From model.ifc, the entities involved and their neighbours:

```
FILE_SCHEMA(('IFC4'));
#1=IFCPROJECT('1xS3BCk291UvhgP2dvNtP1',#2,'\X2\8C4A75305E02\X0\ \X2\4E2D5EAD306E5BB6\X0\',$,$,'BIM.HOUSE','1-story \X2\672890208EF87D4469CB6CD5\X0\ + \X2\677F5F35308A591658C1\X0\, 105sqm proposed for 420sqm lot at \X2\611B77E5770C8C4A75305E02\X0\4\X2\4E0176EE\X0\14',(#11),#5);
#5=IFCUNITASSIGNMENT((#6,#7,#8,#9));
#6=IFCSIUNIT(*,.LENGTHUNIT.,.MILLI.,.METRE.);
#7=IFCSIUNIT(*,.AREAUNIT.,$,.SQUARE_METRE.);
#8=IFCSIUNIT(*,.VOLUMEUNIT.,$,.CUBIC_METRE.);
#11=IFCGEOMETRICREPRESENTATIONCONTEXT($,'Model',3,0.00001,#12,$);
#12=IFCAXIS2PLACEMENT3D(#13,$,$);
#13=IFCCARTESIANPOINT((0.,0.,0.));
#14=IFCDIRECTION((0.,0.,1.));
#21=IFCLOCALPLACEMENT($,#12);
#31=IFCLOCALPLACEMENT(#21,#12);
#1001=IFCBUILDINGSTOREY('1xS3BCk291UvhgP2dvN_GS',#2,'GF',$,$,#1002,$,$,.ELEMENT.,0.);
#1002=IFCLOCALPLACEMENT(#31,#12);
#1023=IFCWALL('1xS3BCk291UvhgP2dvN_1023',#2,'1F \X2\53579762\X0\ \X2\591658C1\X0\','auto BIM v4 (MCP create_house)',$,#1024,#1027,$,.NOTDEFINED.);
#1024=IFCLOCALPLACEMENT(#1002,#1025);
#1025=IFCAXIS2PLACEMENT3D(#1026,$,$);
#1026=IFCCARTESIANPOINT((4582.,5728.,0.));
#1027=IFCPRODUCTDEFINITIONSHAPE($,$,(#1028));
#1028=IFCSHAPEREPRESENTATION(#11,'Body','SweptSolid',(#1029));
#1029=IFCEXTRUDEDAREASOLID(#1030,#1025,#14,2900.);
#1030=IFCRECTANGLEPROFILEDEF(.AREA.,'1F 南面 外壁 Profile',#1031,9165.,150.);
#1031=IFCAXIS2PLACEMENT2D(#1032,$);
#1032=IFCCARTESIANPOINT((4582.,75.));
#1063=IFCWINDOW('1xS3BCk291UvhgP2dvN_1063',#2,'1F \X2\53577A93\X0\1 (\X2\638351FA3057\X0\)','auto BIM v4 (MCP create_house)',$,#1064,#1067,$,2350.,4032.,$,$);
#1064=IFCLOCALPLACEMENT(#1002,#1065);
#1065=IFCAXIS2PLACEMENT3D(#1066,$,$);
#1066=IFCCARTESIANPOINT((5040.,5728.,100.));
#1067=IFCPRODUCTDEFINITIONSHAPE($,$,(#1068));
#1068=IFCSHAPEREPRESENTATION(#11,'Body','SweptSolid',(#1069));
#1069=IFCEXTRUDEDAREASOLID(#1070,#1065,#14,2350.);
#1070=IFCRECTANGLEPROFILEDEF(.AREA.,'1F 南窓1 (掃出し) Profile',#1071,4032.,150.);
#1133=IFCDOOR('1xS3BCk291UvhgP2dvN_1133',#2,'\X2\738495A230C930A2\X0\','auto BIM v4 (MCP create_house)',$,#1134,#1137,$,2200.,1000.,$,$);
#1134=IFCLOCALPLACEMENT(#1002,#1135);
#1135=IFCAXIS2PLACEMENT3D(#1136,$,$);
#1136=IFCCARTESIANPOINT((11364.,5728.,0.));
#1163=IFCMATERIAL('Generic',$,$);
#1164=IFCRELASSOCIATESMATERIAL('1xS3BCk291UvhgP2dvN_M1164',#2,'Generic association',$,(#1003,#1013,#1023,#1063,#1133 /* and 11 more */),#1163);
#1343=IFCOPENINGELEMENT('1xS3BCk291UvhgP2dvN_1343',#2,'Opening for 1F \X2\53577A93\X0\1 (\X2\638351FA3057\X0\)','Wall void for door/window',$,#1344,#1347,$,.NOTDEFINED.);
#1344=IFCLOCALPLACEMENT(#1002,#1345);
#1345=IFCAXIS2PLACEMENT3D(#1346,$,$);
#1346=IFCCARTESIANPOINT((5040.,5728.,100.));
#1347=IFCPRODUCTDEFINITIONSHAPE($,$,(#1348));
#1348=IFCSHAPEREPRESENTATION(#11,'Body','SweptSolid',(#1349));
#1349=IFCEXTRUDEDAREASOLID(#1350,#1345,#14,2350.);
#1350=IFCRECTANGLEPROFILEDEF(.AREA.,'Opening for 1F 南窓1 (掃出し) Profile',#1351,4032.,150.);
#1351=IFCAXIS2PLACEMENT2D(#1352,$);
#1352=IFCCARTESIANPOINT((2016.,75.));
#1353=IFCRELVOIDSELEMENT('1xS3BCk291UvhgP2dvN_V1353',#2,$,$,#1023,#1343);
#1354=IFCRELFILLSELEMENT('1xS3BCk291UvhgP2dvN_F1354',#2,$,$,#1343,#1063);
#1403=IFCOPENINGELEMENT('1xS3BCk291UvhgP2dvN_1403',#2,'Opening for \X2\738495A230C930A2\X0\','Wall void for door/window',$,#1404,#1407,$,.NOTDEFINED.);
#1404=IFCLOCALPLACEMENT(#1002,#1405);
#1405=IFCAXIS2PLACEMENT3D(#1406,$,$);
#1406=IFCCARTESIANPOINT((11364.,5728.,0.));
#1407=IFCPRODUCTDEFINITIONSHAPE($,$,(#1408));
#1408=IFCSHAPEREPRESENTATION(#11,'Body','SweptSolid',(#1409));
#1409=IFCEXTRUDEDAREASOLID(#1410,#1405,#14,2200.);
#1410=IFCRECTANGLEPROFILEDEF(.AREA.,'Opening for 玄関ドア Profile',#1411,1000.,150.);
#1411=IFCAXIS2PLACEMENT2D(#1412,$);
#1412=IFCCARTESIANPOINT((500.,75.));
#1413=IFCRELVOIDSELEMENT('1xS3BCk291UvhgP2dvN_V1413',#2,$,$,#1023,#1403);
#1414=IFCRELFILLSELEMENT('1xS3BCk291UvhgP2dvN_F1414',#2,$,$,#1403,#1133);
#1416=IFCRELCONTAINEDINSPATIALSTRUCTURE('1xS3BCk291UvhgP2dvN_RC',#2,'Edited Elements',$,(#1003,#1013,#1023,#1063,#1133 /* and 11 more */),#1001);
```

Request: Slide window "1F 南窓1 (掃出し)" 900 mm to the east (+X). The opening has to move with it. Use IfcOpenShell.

```python
import ifcopenshell
import ifcopenshell.api.geometry
import ifcopenshell.util.placement
import ifcopenshell.util.unit

model = ifcopenshell.open("model.ifc")
unit_scale = ifcopenshell.util.unit.calculate_unit_scale(model)

window = model.by_guid("1xS3BCk291UvhgP2dvN_1063")
opening = window.FillsVoids[0].RelatingOpeningElement
wall = opening.VoidsElements[0].RelatingBuildingElement

wall_matrix = ifcopenshell.util.placement.get_local_placement(wall.ObjectPlacement)
shift = wall_matrix[:3, 0] * 0.9 / unit_scale
before = ifcopenshell.util.placement.get_local_placement(window.ObjectPlacement)[:3, 3].copy()

# The window is not placed relative to its opening, so move both.
for product in (opening, window):
    matrix = ifcopenshell.util.placement.get_local_placement(product.ObjectPlacement)
    matrix[:3, 3] += shift
    ifcopenshell.api.geometry.edit_object_placement(model, product=product, matrix=matrix, is_si=False)

after = ifcopenshell.util.placement.get_local_placement(window.ObjectPlacement)[:3, 3]
print("window moved by", (after - before).round(3) + 0.0)

model.write("model_edited.ifc")
```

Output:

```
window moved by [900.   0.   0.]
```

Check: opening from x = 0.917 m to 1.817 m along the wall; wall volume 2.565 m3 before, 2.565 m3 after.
